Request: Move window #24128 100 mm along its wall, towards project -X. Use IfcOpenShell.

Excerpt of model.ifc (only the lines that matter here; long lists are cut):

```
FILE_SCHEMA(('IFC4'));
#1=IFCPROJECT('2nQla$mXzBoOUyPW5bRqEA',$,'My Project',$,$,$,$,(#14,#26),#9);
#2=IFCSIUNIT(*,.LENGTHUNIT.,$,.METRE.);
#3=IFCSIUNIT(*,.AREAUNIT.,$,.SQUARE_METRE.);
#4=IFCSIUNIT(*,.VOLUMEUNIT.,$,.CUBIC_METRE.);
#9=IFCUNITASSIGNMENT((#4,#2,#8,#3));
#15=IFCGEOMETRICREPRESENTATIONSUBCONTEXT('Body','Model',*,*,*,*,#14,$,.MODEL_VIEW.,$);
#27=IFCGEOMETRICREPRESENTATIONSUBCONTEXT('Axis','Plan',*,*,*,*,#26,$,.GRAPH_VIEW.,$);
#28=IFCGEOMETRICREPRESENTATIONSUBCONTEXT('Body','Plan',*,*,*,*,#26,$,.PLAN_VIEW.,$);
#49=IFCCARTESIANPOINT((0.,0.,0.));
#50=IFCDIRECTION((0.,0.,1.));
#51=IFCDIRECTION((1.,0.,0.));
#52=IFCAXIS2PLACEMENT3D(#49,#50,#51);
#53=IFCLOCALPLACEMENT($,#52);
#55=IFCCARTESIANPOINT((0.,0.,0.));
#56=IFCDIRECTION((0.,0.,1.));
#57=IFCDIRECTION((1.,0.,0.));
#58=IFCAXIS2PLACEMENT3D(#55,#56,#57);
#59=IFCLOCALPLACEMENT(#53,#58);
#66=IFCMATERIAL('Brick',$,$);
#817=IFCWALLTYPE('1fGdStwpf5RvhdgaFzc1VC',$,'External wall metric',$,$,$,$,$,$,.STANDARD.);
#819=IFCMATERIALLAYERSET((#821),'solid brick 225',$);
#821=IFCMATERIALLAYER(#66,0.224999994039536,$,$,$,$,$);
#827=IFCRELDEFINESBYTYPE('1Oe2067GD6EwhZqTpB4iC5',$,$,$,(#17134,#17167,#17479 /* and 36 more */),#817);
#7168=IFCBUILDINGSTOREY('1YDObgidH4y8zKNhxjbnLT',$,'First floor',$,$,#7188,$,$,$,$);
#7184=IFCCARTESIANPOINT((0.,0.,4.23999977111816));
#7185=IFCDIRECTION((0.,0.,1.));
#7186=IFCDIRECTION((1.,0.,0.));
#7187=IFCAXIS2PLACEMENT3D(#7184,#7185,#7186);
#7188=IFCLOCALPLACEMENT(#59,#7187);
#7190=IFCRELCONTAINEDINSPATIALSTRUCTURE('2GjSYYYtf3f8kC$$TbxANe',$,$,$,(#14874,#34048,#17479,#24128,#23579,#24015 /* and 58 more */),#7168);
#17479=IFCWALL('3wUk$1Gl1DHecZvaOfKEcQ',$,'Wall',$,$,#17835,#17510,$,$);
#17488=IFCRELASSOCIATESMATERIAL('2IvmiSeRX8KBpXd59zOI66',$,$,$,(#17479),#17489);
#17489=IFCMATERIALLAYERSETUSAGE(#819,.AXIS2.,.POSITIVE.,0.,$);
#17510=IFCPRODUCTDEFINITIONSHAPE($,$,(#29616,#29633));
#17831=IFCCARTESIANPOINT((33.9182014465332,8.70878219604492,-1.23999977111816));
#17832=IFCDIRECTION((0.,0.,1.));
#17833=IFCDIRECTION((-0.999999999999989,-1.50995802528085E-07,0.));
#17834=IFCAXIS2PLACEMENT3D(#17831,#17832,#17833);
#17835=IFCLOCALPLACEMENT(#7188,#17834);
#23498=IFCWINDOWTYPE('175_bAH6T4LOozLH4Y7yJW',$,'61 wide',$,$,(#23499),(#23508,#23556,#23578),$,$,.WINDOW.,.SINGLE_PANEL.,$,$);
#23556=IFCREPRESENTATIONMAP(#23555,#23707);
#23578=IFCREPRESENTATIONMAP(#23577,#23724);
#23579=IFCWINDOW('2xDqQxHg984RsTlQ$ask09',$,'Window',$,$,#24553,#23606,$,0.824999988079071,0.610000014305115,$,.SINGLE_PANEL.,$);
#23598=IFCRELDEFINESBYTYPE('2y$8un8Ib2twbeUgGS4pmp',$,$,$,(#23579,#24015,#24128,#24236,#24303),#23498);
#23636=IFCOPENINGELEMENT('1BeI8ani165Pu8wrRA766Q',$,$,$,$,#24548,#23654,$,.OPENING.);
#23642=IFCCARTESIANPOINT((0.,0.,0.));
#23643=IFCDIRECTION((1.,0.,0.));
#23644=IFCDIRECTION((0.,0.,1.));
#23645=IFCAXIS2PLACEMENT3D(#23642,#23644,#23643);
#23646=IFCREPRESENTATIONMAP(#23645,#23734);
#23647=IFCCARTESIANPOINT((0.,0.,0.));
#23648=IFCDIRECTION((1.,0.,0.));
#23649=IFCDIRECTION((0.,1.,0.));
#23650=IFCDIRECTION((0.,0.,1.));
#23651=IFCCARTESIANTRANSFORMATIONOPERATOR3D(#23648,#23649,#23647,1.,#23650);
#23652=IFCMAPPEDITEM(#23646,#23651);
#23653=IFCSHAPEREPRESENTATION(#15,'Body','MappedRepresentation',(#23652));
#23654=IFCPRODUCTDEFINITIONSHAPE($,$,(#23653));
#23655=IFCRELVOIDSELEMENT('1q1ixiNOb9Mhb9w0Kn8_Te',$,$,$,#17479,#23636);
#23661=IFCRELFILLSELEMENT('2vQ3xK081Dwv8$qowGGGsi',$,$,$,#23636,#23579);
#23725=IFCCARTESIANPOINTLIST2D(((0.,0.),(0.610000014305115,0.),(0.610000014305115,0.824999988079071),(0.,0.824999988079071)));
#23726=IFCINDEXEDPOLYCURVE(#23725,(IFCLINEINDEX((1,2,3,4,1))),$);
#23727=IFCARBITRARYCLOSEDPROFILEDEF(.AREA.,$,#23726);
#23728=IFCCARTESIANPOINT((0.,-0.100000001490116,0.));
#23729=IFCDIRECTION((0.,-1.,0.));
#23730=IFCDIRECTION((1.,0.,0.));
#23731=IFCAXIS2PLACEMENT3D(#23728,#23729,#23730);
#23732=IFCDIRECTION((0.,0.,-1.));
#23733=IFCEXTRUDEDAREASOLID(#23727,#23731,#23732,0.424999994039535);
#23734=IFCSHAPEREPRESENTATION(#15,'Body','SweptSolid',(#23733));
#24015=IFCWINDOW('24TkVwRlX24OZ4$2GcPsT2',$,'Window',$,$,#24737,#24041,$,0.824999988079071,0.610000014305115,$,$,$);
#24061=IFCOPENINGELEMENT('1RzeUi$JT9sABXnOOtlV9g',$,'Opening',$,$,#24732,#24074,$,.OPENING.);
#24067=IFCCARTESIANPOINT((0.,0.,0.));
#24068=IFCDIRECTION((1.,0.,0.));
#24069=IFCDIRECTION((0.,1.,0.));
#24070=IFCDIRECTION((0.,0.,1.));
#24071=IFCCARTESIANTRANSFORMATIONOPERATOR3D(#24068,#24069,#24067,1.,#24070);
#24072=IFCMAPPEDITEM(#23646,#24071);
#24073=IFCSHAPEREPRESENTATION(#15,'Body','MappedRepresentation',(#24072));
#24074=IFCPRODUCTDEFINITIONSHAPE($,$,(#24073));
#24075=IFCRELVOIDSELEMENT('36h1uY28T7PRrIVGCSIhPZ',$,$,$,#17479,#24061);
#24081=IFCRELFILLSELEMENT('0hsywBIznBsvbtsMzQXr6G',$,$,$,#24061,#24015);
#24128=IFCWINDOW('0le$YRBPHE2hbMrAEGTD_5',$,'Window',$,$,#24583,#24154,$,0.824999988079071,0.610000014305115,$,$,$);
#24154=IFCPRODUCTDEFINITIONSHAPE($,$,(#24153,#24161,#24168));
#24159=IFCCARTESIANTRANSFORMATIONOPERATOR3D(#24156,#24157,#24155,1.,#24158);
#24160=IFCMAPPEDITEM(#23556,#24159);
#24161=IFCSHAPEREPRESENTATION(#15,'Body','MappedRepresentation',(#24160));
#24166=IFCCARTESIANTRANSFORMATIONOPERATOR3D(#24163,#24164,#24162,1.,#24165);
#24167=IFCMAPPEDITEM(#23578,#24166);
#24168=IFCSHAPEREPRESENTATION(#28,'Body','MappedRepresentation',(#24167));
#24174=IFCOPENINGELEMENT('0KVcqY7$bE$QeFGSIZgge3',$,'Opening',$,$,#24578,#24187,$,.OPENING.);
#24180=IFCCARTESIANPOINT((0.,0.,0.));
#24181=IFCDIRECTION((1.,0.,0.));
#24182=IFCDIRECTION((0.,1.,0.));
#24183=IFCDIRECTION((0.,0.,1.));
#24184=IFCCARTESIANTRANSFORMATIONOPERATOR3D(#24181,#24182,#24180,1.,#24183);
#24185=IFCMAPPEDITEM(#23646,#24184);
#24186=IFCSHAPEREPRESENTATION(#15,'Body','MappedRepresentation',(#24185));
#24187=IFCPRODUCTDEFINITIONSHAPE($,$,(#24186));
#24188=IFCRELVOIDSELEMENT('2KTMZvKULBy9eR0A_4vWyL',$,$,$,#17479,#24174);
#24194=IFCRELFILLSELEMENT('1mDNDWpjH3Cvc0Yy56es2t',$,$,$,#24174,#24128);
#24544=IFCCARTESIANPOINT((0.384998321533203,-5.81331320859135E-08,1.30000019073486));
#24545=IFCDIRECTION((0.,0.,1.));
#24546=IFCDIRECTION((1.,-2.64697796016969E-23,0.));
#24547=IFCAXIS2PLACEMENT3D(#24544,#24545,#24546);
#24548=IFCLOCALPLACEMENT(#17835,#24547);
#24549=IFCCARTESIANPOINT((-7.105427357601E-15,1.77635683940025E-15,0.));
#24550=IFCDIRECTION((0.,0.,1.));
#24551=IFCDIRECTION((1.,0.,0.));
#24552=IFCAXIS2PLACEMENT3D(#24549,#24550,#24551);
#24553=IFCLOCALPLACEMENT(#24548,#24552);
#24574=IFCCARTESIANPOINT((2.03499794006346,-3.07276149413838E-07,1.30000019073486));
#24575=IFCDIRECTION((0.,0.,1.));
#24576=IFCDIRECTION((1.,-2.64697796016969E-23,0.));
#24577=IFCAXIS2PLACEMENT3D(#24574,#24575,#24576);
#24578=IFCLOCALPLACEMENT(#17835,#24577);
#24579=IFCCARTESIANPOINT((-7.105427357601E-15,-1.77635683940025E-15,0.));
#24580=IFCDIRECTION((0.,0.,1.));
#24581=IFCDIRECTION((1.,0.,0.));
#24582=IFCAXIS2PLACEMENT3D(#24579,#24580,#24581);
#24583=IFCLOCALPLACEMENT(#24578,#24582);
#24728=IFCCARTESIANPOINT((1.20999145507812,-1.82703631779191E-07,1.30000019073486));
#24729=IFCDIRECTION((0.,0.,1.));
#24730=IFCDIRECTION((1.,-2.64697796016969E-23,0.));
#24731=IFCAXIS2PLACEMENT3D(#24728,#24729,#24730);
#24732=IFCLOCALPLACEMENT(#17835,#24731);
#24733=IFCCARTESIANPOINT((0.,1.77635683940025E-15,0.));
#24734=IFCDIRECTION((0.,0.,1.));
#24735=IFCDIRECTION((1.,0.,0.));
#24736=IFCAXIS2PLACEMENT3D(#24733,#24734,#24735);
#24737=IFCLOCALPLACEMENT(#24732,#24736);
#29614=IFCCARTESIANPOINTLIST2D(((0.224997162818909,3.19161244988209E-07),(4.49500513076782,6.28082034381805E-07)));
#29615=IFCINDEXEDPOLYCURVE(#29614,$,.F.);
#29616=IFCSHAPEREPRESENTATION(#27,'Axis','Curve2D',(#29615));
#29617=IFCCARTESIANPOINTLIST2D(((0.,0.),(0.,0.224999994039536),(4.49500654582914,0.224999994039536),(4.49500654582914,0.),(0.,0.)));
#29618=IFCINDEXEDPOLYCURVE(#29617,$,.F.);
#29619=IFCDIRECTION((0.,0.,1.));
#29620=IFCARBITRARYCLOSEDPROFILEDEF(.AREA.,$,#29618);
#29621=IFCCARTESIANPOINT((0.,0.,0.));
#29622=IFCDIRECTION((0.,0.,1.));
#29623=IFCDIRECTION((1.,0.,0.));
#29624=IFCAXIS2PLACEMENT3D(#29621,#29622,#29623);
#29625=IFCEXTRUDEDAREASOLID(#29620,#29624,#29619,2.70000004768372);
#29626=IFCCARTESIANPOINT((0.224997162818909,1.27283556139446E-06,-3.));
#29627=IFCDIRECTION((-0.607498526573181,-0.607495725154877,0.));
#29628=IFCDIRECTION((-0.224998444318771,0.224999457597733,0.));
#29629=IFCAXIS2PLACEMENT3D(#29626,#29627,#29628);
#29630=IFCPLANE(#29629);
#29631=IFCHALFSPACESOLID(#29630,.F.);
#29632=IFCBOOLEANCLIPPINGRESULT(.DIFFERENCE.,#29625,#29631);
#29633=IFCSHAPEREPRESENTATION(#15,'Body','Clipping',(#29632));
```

```python
import ifcopenshell
import ifcopenshell.api.geometry
import ifcopenshell.util.placement
import ifcopenshell.util.unit

model = ifcopenshell.open("model.ifc")
unit_scale = ifcopenshell.util.unit.calculate_unit_scale(model)

window = model.by_guid("0le$YRBPHE2hbMrAEGTD_5")
opening = window.FillsVoids[0].RelatingOpeningElement
wall = opening.VoidsElements[0].RelatingBuildingElement

wall_matrix = ifcopenshell.util.placement.get_local_placement(wall.ObjectPlacement)
shift = wall_matrix[:3, 0] * 0.1 / unit_scale
before = ifcopenshell.util.placement.get_local_placement(window.ObjectPlacement)[:3, 3].copy()

# The window is placed relative to its opening, so it follows when the opening moves.
matrix = ifcopenshell.util.placement.get_local_placement(opening.ObjectPlacement)
matrix[:3, 3] += shift
ifcopenshell.api.geometry.edit_object_placement(
    model, product=opening, matrix=matrix, is_si=False, should_transform_children=True
)

after = ifcopenshell.util.placement.get_local_placement(window.ObjectPlacement)[:3, 3]
print("window moved by", (after - before).round(3) + 0.0)

model.write("model_edited.ifc")
```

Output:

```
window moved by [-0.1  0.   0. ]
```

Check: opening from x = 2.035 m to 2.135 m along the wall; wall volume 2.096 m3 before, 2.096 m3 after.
